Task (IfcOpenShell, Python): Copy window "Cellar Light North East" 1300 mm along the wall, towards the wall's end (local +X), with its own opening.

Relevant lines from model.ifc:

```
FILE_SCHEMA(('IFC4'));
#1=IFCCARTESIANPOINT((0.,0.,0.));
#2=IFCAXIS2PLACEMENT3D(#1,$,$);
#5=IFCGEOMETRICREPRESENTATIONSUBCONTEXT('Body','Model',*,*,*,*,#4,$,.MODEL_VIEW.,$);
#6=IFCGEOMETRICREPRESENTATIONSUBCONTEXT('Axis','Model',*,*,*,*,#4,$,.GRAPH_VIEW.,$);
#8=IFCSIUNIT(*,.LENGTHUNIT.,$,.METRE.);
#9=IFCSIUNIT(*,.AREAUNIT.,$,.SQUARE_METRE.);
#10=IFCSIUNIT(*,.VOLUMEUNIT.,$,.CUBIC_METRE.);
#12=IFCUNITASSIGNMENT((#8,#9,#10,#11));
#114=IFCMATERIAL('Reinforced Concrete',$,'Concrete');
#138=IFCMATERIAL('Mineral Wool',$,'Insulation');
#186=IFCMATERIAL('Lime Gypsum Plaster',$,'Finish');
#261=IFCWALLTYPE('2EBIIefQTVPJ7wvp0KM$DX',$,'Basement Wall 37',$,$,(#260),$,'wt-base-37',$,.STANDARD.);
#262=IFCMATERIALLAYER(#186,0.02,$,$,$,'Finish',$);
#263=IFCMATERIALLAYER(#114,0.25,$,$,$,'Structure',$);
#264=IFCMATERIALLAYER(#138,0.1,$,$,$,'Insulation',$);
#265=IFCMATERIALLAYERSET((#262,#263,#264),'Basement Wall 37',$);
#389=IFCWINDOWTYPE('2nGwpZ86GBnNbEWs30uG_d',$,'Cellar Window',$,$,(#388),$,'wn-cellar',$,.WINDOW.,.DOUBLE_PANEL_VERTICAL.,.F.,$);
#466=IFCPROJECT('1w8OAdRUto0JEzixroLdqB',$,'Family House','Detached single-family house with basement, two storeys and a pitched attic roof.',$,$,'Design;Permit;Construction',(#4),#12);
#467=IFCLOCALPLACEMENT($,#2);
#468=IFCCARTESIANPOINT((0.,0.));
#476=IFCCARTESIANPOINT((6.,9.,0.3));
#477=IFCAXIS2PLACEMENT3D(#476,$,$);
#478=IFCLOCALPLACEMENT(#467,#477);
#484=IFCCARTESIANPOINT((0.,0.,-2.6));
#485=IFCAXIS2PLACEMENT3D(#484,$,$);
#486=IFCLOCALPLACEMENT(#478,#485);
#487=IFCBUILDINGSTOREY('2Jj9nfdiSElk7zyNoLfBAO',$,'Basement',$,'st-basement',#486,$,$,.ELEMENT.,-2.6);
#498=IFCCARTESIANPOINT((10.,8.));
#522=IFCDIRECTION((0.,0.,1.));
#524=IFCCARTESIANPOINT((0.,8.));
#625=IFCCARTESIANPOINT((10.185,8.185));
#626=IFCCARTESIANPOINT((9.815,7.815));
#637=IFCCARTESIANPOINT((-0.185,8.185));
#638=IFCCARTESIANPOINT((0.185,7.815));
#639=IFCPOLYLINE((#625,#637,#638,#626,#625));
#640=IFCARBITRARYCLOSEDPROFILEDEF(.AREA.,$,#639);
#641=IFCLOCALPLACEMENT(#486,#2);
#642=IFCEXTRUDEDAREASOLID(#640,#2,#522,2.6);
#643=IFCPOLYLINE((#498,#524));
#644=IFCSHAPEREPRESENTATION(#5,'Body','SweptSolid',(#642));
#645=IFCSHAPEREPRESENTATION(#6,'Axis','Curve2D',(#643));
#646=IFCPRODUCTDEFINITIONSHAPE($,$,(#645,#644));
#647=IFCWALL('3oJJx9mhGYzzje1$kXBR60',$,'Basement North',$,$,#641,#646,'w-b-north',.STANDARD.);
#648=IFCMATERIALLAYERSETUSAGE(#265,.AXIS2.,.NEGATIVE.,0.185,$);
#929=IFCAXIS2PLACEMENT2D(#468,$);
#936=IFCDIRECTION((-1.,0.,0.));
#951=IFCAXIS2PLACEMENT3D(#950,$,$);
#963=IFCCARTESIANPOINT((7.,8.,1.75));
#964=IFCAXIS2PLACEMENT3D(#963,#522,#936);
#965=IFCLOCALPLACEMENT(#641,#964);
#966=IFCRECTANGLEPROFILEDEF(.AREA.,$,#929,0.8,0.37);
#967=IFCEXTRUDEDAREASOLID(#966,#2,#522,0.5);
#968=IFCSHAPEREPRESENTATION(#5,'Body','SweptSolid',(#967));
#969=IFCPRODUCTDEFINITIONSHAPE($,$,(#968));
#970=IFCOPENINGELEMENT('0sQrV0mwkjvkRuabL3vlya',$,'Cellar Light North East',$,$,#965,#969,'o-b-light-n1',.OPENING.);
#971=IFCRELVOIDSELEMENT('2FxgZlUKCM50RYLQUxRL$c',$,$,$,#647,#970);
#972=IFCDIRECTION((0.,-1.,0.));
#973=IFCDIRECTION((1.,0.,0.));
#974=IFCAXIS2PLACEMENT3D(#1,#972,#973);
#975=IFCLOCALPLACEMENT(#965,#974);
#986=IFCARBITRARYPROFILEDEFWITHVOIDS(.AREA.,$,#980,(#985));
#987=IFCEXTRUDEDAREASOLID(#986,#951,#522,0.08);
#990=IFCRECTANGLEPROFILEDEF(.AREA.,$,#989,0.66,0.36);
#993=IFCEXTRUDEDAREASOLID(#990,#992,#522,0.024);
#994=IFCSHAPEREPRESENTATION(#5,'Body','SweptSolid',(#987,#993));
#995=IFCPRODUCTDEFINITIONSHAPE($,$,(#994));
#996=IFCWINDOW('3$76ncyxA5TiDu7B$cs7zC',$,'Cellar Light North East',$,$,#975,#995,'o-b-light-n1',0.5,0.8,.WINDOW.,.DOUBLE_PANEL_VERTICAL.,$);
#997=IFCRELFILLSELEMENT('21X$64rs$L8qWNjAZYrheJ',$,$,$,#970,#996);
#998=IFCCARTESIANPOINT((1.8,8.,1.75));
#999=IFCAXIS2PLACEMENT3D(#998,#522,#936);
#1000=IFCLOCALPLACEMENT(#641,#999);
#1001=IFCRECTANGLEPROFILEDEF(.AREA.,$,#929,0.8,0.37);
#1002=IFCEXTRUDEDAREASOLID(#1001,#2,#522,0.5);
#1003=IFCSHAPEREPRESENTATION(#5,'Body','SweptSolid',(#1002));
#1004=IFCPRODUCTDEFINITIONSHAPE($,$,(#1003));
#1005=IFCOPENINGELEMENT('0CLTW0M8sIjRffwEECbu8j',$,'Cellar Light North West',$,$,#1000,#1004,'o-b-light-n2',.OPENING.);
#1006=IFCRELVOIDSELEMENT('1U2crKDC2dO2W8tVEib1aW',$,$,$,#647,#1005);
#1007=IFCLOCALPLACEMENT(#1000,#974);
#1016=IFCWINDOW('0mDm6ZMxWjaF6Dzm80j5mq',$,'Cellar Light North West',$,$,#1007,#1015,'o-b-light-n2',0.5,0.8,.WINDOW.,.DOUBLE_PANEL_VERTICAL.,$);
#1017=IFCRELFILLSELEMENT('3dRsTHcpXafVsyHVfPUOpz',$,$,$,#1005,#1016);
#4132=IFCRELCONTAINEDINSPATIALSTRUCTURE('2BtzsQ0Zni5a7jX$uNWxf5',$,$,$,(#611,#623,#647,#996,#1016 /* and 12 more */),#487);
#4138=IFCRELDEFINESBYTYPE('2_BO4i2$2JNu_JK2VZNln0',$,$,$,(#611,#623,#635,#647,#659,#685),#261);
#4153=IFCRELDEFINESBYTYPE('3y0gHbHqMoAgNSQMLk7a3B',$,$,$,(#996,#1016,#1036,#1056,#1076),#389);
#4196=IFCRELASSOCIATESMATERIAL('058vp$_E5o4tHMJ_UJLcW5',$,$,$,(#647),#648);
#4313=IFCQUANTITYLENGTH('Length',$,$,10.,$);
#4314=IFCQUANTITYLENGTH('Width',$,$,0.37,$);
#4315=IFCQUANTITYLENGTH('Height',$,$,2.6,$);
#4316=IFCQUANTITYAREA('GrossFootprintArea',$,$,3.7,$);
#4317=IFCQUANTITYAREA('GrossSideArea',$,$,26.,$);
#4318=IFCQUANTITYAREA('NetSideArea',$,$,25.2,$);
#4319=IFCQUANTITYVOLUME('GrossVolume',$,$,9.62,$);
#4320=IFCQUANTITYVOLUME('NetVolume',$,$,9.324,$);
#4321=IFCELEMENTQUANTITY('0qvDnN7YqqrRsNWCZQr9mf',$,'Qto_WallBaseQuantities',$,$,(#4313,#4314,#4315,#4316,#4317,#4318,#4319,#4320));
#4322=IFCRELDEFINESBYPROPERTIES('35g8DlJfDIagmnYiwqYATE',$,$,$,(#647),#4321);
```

```python
import ifcopenshell
import ifcopenshell.api.feature
import ifcopenshell.api.geometry
import ifcopenshell.api.pset
import ifcopenshell.api.root
import ifcopenshell.geom
import ifcopenshell.util.element
import ifcopenshell.util.placement
import ifcopenshell.util.shape
import ifcopenshell.util.unit

model = ifcopenshell.open("model.ifc")
unit_scale = ifcopenshell.util.unit.calculate_unit_scale(model)
area_scale = ifcopenshell.util.unit.calculate_unit_scale(model, "AREAUNIT")
volume_scale = ifcopenshell.util.unit.calculate_unit_scale(model, "VOLUMEUNIT")
settings = ifcopenshell.geom.settings()


def volume(element):
    """Net volume in cubic metres, openings subtracted."""
    shape = ifcopenshell.geom.create_shape(settings, element)
    return ifcopenshell.util.shape.get_volume(shape.geometry)


window = model.by_guid("3$76ncyxA5TiDu7B$cs7zC")
opening = window.FillsVoids[0].RelatingOpeningElement
wall = opening.VoidsElements[0].RelatingBuildingElement
before = volume(wall)
shift = ifcopenshell.util.placement.get_local_placement(wall.ObjectPlacement)[:3, 0] * 1.3 / unit_scale

# copy_class copies the void relationship, type, container and properties, but no geometry.
new_opening = ifcopenshell.api.root.copy_class(model, product=opening)
new_opening.Representation = ifcopenshell.util.element.copy_deep(
    model, opening.Representation, exclude=["IfcGeometricRepresentationContext", "IfcRepresentationMap"]
)
new_opening.Tag = None
new_window = ifcopenshell.api.root.copy_class(model, product=window)
new_window.Representation = ifcopenshell.util.element.copy_deep(
    model, window.Representation, exclude=["IfcGeometricRepresentationContext", "IfcRepresentationMap"]
)
new_window.Tag = None
ifcopenshell.api.feature.add_filling(model, opening=new_opening, element=new_window)

for old, new in ((opening, new_opening), (window, new_window)):
    matrix = ifcopenshell.util.placement.get_local_placement(old.ObjectPlacement)
    matrix[:3, 3] += shift
    ifcopenshell.api.geometry.edit_object_placement(model, product=new, matrix=matrix, is_si=False)

after = volume(wall)
thickness = 0.37  # wall thickness in metres

# Update the wall's stored quantities.
qto = model.by_id(ifcopenshell.util.element.get_pset(wall, "Qto_WallBaseQuantities", should_inherit=False)["id"])
ifcopenshell.api.pset.edit_qto(model, qto=qto, properties={
    "NetSideArea": after / thickness / area_scale,
    "NetVolume": after / volume_scale,
})

print(f"wall volume {before:.3f} -> {after:.3f} m3")

model.write("model_edited.ifc")
```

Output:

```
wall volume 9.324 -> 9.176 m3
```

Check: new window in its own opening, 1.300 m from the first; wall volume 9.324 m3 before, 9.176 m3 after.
